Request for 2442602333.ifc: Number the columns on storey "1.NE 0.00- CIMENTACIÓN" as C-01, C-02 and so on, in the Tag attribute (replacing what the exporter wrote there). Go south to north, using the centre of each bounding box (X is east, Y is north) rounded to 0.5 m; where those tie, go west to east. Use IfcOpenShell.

First a look at what the model holds.

```python
import ifcopenshell
import ifcopenshell.util.element
import ifcopenshell.util.placement

model = ifcopenshell.open("2442602333.ifc")
print(model.schema)
storey = next(s for s in model.by_type("IfcBuildingStorey") if s.Name == "1.NE 0.00- CIMENTACIÓN")
columns = [e for e in ifcopenshell.util.element.get_decomposition(storey) if e.is_a("IfcColumn")]
for e in sorted(columns, key=lambda e: e.id()):
    origin = ifcopenshell.util.placement.get_local_placement(e.ObjectPlacement)[:3, 3]
    print(e.id(), e.Tag, e.Name, origin.round(2) + 0.0, sep=" | ")
```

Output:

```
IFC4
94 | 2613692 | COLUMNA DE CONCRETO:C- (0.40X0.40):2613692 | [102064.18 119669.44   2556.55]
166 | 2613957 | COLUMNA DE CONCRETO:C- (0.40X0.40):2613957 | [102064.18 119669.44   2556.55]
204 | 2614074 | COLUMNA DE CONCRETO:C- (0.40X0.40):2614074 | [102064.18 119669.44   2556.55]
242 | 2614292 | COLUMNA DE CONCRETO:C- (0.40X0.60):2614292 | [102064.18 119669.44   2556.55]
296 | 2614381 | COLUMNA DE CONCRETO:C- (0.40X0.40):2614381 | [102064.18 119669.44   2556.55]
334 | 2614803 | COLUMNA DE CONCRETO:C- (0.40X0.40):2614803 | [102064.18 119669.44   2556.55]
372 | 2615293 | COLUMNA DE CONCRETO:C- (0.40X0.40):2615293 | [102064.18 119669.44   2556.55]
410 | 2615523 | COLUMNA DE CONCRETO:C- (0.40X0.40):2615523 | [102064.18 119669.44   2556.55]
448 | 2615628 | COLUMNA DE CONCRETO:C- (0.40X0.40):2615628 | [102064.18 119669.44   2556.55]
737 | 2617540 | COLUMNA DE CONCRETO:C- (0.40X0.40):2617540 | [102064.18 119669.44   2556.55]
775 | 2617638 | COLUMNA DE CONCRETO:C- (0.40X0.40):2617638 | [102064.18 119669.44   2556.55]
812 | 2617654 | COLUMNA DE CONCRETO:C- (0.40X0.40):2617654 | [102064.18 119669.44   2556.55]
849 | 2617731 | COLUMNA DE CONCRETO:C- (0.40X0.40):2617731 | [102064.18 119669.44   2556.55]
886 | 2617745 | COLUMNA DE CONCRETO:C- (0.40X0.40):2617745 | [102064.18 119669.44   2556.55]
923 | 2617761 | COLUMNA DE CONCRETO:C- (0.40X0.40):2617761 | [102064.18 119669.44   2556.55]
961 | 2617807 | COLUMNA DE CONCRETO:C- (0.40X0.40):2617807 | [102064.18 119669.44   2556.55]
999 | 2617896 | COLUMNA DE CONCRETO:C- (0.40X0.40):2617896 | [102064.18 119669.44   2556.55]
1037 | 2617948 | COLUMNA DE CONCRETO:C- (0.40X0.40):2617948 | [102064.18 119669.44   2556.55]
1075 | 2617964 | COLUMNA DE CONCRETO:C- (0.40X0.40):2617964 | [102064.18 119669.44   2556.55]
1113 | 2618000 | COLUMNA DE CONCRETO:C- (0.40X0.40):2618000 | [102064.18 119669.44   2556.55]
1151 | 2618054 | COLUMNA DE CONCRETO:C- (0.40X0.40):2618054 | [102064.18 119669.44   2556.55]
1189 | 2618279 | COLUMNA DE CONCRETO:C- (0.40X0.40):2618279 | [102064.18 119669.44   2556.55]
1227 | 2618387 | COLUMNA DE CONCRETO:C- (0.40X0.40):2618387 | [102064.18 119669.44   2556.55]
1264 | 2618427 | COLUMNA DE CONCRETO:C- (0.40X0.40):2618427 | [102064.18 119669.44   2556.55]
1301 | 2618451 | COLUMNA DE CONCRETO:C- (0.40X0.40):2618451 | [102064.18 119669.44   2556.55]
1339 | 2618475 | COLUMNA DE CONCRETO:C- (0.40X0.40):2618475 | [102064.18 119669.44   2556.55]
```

```python
import ifcopenshell
import ifcopenshell.geom
import ifcopenshell.util.element
import ifcopenshell.util.shape

model = ifcopenshell.open("2442602333.ifc")
settings = ifcopenshell.geom.settings()
settings.set("use-world-coords", True)


def centre(element):
    shape = ifcopenshell.geom.create_shape(settings, element)
    return ifcopenshell.util.shape.get_bbox_centroid(shape.geometry)


storey = next(s for s in model.by_type("IfcBuildingStorey") if s.Name == "1.NE 0.00- CIMENTACIÓN")
columns = [e for e in ifcopenshell.util.element.get_decomposition(storey) if e.is_a("IfcColumn")]

# Insertion points can sit at a corner or the storey origin, so sort by the geometry (in metres).
centres = {e: centre(e) for e in columns}
columns.sort(key=lambda e: (round(centres[e][1] / 0.5), centres[e][0]))

for i, e in enumerate(columns, start=1):
    number = f"C-{i:02d}"
    e.Tag = number
    print(e.id(), number)

model.write("2442602333-out.ifc")
```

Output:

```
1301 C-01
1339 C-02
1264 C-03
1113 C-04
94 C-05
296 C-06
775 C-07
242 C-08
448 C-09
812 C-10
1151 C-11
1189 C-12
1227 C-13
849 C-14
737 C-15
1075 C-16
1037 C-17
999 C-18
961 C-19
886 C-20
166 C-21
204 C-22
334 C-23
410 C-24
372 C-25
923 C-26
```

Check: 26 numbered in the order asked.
